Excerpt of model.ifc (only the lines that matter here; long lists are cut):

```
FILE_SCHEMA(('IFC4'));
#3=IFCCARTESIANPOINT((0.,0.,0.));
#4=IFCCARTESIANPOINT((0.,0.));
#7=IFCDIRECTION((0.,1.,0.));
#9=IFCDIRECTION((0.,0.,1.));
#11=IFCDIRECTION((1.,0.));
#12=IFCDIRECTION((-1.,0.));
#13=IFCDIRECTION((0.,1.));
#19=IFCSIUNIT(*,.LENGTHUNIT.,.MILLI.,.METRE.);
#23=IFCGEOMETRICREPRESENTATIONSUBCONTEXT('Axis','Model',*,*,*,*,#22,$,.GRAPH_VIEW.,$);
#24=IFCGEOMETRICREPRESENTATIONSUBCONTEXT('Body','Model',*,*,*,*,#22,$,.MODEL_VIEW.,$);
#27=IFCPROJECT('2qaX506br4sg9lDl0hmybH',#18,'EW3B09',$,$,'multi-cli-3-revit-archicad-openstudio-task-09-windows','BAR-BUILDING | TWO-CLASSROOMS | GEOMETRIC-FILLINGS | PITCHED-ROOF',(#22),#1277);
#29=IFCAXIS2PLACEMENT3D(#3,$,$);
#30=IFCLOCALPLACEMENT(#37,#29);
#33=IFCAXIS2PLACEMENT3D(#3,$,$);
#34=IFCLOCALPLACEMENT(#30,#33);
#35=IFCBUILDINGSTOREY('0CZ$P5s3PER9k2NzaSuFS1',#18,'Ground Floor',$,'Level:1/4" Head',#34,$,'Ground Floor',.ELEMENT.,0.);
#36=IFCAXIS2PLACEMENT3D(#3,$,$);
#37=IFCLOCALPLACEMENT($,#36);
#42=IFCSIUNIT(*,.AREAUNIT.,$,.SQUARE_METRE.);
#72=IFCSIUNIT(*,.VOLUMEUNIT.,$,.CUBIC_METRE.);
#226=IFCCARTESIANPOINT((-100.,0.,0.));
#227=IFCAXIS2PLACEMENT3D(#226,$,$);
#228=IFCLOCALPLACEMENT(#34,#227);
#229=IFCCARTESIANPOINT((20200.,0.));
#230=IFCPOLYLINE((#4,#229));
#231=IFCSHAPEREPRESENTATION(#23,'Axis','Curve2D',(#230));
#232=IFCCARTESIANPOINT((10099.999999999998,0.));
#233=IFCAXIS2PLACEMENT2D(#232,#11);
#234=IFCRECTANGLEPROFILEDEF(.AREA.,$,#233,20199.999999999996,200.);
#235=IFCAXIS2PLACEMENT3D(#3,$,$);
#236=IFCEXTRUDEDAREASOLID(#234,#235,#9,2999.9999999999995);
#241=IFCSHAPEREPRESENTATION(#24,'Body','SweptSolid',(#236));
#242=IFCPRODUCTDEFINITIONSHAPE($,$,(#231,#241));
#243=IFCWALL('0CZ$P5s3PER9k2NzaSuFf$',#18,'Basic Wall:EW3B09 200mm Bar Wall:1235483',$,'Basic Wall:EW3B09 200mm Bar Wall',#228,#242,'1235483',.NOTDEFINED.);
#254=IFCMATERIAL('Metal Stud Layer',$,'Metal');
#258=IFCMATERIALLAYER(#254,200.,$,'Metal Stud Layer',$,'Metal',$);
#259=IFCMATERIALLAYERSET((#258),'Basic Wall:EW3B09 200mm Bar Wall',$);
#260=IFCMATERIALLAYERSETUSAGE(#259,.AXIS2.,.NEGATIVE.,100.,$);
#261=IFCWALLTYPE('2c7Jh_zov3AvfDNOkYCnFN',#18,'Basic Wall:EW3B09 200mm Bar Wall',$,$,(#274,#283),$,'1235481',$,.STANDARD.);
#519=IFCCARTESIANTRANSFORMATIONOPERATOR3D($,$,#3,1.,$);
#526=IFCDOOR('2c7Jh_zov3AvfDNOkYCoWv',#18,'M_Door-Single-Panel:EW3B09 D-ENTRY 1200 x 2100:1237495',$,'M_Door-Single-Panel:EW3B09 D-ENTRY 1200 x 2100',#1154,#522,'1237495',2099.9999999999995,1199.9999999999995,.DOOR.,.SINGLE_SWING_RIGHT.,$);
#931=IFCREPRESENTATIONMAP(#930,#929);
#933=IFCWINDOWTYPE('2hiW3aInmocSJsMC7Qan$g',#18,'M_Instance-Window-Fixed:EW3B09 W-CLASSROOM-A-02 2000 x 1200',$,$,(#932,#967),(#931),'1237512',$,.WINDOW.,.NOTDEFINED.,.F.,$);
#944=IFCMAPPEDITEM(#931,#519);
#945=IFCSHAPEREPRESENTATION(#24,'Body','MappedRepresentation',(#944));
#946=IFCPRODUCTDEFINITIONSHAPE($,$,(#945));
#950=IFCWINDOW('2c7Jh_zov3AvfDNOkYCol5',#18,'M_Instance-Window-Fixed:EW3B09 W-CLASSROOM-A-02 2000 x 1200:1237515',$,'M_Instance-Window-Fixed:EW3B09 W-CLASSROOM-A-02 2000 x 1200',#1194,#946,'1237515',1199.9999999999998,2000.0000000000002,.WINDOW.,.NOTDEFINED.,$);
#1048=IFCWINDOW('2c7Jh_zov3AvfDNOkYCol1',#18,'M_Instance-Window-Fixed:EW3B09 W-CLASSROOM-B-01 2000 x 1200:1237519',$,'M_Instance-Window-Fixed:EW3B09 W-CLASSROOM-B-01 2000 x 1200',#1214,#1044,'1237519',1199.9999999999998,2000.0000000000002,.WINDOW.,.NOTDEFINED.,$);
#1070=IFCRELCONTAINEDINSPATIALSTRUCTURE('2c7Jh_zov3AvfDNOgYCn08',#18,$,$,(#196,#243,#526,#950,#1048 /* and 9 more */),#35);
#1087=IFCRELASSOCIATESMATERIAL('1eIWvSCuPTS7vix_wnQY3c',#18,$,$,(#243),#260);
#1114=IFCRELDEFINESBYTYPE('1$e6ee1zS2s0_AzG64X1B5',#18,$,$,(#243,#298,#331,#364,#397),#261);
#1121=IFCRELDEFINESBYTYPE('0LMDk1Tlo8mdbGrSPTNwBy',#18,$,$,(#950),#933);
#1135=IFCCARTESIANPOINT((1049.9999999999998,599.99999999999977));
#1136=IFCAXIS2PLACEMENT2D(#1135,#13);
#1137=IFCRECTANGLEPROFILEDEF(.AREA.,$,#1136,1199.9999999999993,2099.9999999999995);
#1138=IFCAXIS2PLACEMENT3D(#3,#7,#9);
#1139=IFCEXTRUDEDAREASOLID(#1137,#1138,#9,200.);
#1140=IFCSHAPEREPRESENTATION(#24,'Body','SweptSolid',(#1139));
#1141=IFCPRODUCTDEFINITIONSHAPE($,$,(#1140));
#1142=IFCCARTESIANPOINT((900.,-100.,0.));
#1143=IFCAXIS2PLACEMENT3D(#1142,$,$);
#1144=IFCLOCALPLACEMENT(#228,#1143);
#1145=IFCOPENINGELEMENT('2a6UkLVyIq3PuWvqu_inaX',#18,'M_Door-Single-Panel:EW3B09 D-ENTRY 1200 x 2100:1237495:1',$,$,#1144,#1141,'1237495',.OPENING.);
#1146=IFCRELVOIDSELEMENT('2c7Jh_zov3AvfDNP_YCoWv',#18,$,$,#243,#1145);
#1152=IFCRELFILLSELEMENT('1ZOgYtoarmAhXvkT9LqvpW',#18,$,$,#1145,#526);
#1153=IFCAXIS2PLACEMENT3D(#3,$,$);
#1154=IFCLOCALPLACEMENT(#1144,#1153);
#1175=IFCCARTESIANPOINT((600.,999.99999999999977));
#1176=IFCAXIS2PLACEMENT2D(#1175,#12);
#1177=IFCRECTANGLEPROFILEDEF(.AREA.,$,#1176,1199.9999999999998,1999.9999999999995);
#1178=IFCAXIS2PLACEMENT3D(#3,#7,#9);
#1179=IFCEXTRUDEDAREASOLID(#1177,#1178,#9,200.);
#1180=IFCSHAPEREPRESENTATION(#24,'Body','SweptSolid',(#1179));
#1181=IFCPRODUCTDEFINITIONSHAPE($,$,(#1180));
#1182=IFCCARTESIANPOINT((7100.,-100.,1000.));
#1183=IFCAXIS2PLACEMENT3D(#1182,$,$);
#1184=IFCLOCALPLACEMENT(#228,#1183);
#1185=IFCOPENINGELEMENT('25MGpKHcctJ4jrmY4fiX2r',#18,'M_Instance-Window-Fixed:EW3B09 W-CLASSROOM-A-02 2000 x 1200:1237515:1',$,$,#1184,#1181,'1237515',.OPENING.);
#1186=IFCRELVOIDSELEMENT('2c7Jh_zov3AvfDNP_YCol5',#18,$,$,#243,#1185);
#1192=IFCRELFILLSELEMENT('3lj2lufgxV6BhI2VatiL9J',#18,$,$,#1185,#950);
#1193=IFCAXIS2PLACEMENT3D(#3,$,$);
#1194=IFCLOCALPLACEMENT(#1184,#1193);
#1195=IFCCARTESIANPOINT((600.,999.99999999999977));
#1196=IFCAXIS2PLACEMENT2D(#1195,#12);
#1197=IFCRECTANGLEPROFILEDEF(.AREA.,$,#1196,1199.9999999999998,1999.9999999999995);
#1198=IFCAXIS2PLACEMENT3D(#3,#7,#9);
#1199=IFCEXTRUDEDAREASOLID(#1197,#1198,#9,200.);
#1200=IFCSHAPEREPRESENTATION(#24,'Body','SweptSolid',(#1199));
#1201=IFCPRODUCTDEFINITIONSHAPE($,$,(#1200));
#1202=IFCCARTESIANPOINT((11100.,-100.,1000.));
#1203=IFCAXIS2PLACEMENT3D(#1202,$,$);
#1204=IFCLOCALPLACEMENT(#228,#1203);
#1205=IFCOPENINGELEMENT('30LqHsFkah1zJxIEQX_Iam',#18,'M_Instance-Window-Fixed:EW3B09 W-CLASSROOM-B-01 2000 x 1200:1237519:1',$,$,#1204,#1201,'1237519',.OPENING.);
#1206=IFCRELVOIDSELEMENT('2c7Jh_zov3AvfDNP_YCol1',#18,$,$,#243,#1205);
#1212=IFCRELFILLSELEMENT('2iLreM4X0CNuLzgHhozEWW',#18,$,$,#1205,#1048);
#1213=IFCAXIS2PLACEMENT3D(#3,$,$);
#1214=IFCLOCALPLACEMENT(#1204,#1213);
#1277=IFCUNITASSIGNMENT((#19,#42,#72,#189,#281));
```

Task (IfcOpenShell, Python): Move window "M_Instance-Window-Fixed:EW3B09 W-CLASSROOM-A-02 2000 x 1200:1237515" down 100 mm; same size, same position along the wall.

```python
import numpy as np
import ifcopenshell
import ifcopenshell.api.geometry
import ifcopenshell.util.placement
import ifcopenshell.util.unit

model = ifcopenshell.open("model.ifc")
unit_scale = ifcopenshell.util.unit.calculate_unit_scale(model)

window = model.by_guid("2c7Jh_zov3AvfDNOkYCol5")
opening = window.FillsVoids[0].RelatingOpeningElement
dz = -100.0

shift = np.array([0.0, 0.0, dz])
# The window is placed relative to its opening, so it follows when the opening moves.
matrix = ifcopenshell.util.placement.get_local_placement(opening.ObjectPlacement)
matrix[:3, 3] += shift
ifcopenshell.api.geometry.edit_object_placement(
    model, product=opening, matrix=matrix, is_si=False, should_transform_children=True
)

print(f"moved by {dz * unit_scale:+.3f} m")

model.write("model-out.ifc")
```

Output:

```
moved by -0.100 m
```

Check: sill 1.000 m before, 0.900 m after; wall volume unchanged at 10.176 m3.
